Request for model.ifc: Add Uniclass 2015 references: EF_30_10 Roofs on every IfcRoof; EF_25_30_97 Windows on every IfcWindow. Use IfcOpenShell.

First a look at what the model holds.

```python
import ifcopenshell

model = ifcopenshell.open("model.ifc")
print(model.schema)
print("classifications:", [c.Name for c in model.by_type("IfcClassification")])
for ifc_class in ("IfcDoor", "IfcRoof", "IfcStair", "IfcWall", "IfcWindow"):
    print(ifc_class, len(model.by_type(ifc_class)))
```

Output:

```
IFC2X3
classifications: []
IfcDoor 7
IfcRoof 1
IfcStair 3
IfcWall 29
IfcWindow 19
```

```python
import ifcopenshell
import ifcopenshell.api.classification

model = ifcopenshell.open("model.ifc")

# IFC2X3 requires Source and Edition and has no link from the project to the system.
system = model.create_entity("IfcClassification", Source="NBS", Edition="2015", Name="Uniclass 2015")

codes = {
    "IfcRoof": ("EF_30_10", "Roofs"),
    "IfcWindow": ("EF_25_30_97", "Windows"),
}
for ifc_class, (code, name) in codes.items():
    products = model.by_type(ifc_class)
    ifcopenshell.api.classification.add_reference(
        model, products=products, classification=system, identification=code, name=name
    )
    print(code, len(products))

model.write("model_v2.ifc")
```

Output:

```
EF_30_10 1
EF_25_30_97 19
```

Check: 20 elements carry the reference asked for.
